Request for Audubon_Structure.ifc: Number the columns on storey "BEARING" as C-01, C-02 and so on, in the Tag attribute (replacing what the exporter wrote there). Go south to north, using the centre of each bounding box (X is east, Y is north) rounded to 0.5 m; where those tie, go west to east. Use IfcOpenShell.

First a look at what the model holds.

```python
import ifcopenshell
import ifcopenshell.util.element
import ifcopenshell.util.placement

model = ifcopenshell.open("Audubon_Structure.ifc")
print(model.schema)
storey = next(s for s in model.by_type("IfcBuildingStorey") if s.Name == "BEARING")
columns = [e for e in ifcopenshell.util.element.get_decomposition(storey) if e.is_a("IfcColumn")]
for e in sorted(columns, key=lambda e: e.id()):
    origin = ifcopenshell.util.placement.get_local_placement(e.ObjectPlacement)[:3, 3]
    print(e.id(), e.Tag, e.Name, origin.round(2) + 0.0, sep=" | ")
```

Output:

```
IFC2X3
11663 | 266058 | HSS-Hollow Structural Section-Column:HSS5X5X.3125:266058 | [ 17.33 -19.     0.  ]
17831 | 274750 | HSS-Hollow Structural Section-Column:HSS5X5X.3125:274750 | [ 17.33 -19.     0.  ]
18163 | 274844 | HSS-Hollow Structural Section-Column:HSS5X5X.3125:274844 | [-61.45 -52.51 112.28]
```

```python
import ifcopenshell
import ifcopenshell.geom
import ifcopenshell.util.element
import ifcopenshell.util.shape

model = ifcopenshell.open("Audubon_Structure.ifc")
settings = ifcopenshell.geom.settings()
settings.set("use-world-coords", True)


def centre(element):
    shape = ifcopenshell.geom.create_shape(settings, element)
    return ifcopenshell.util.shape.get_bbox_centroid(shape.geometry)


storey = next(s for s in model.by_type("IfcBuildingStorey") if s.Name == "BEARING")
columns = [e for e in ifcopenshell.util.element.get_decomposition(storey) if e.is_a("IfcColumn")]

# Insertion points can sit at a corner or the storey origin, so sort by the geometry (in metres).
centres = {e: centre(e) for e in columns}
columns.sort(key=lambda e: (round(centres[e][1] / 0.5), centres[e][0]))

for i, e in enumerate(columns, start=1):
    number = f"C-{i:02d}"
    e.Tag = number
    print(e.id(), number)

model.write("Audubon_Structure_v2.ifc")
```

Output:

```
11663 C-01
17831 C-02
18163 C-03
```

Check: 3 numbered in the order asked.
